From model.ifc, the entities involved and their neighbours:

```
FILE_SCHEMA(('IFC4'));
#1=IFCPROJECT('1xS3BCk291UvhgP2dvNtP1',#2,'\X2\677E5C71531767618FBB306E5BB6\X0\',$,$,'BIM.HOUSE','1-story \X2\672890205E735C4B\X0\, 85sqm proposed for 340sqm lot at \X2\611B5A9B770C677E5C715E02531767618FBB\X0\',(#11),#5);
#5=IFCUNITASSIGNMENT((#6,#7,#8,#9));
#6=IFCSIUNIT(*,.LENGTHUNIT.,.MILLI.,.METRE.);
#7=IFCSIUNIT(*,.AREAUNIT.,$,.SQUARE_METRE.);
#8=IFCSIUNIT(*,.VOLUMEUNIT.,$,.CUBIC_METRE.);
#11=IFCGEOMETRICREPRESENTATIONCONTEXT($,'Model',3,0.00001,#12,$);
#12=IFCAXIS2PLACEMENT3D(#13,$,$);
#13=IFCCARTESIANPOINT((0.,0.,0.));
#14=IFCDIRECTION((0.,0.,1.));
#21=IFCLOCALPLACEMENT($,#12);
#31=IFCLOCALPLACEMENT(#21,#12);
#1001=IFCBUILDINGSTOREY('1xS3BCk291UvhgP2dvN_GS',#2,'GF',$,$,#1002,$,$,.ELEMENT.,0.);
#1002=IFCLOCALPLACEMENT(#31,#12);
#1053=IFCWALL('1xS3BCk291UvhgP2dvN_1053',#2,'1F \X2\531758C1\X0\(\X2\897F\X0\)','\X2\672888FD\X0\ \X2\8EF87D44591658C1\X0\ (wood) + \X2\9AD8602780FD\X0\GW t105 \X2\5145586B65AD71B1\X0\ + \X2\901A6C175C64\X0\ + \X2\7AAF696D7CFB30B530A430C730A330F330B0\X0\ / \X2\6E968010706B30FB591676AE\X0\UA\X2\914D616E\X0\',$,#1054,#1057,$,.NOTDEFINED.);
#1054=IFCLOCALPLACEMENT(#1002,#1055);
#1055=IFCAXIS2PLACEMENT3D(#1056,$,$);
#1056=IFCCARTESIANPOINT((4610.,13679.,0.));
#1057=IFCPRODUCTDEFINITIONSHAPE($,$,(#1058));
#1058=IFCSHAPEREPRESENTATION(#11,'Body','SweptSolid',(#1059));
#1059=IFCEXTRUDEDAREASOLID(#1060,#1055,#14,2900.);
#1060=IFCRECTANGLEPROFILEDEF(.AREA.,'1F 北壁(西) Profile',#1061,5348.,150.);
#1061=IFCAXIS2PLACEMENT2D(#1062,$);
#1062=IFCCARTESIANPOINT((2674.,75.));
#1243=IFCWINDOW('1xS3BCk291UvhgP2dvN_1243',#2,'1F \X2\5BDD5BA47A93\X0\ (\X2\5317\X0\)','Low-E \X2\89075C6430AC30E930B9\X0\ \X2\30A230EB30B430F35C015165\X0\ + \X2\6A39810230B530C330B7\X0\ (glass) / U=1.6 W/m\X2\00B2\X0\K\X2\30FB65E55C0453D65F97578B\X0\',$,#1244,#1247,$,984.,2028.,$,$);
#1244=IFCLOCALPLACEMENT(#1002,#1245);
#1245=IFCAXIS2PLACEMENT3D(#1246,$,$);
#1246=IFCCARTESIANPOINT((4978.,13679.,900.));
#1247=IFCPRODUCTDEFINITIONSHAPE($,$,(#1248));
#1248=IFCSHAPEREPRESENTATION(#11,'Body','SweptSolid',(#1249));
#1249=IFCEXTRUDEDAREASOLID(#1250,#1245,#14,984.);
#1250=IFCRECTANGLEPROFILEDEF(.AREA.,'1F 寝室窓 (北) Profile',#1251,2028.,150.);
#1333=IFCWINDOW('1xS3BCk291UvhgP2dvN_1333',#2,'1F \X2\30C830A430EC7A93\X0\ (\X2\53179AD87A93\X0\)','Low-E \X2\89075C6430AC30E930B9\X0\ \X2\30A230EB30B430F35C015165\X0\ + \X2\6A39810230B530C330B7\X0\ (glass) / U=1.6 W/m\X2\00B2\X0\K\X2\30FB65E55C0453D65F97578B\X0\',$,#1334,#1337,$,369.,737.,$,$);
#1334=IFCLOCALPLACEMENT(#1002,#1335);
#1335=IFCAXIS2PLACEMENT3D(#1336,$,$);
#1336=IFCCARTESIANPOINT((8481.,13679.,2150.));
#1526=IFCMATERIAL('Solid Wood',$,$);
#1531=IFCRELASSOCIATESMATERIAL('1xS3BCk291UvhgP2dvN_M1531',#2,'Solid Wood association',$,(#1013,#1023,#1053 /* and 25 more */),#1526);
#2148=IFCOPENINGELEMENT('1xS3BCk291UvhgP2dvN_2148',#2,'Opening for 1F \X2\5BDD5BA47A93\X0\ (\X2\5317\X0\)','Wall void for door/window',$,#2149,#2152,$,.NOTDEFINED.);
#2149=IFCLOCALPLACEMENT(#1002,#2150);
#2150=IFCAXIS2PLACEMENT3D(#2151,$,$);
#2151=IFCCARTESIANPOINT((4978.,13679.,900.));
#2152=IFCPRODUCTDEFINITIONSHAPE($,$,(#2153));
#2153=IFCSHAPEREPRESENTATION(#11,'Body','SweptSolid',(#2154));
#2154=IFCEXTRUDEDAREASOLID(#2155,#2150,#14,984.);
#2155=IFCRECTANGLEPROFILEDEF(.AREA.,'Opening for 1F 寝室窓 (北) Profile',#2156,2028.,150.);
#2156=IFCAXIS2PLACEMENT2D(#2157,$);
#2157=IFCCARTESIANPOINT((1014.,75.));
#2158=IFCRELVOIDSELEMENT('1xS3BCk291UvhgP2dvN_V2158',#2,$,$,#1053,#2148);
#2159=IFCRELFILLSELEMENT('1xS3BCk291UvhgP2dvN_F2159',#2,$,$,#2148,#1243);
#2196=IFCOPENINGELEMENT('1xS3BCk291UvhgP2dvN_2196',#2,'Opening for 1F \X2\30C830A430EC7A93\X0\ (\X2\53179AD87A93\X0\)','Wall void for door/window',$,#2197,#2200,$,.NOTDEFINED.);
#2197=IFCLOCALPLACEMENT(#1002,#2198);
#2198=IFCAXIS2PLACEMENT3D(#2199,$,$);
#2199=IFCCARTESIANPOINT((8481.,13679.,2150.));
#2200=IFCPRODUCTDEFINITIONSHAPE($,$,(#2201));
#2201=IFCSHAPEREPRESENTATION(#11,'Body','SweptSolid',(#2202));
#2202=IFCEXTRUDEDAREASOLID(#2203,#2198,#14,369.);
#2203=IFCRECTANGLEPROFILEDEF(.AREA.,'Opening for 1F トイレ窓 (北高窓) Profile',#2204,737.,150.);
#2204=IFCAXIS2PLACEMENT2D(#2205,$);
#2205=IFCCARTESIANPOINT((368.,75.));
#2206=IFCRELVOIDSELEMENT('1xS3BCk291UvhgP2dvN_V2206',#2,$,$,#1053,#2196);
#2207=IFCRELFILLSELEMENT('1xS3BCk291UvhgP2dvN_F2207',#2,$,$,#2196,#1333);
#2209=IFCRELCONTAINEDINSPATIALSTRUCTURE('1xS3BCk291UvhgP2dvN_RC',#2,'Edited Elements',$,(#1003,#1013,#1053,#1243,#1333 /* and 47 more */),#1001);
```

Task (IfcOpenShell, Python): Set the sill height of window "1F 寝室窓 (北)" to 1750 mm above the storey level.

```python
import numpy as np
import ifcopenshell
import ifcopenshell.api.geometry
import ifcopenshell.geom
import ifcopenshell.util.element
import ifcopenshell.util.placement
import ifcopenshell.util.shape
import ifcopenshell.util.unit

model = ifcopenshell.open("model.ifc")
unit_scale = ifcopenshell.util.unit.calculate_unit_scale(model)

window = model.by_guid("1xS3BCk291UvhgP2dvN_1243")
opening = window.FillsVoids[0].RelatingOpeningElement
storey = ifcopenshell.util.element.get_container(window, ifc_class="IfcBuildingStorey")
level = ifcopenshell.util.placement.get_local_placement(storey.ObjectPlacement)[2, 3]

# The opening's origin need not be at the sill, so measure its lowest point.
shape = ifcopenshell.geom.create_shape(ifcopenshell.geom.settings(), opening)
bottom = ifcopenshell.util.shape.get_shape_bottom_elevation(shape, shape.geometry) / unit_scale
dz = level + 1.75 / unit_scale - bottom

shift = np.array([0.0, 0.0, dz])
# The window is not placed relative to its opening, so move both.
for product in (opening, window):
    matrix = ifcopenshell.util.placement.get_local_placement(product.ObjectPlacement)
    matrix[:3, 3] += shift
    ifcopenshell.api.geometry.edit_object_placement(model, product=product, matrix=matrix, is_si=False)

print(f"moved by {dz * unit_scale:+.3f} m")

model.write("model_rev.ifc")
```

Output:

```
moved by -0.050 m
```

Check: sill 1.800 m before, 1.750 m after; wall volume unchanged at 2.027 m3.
